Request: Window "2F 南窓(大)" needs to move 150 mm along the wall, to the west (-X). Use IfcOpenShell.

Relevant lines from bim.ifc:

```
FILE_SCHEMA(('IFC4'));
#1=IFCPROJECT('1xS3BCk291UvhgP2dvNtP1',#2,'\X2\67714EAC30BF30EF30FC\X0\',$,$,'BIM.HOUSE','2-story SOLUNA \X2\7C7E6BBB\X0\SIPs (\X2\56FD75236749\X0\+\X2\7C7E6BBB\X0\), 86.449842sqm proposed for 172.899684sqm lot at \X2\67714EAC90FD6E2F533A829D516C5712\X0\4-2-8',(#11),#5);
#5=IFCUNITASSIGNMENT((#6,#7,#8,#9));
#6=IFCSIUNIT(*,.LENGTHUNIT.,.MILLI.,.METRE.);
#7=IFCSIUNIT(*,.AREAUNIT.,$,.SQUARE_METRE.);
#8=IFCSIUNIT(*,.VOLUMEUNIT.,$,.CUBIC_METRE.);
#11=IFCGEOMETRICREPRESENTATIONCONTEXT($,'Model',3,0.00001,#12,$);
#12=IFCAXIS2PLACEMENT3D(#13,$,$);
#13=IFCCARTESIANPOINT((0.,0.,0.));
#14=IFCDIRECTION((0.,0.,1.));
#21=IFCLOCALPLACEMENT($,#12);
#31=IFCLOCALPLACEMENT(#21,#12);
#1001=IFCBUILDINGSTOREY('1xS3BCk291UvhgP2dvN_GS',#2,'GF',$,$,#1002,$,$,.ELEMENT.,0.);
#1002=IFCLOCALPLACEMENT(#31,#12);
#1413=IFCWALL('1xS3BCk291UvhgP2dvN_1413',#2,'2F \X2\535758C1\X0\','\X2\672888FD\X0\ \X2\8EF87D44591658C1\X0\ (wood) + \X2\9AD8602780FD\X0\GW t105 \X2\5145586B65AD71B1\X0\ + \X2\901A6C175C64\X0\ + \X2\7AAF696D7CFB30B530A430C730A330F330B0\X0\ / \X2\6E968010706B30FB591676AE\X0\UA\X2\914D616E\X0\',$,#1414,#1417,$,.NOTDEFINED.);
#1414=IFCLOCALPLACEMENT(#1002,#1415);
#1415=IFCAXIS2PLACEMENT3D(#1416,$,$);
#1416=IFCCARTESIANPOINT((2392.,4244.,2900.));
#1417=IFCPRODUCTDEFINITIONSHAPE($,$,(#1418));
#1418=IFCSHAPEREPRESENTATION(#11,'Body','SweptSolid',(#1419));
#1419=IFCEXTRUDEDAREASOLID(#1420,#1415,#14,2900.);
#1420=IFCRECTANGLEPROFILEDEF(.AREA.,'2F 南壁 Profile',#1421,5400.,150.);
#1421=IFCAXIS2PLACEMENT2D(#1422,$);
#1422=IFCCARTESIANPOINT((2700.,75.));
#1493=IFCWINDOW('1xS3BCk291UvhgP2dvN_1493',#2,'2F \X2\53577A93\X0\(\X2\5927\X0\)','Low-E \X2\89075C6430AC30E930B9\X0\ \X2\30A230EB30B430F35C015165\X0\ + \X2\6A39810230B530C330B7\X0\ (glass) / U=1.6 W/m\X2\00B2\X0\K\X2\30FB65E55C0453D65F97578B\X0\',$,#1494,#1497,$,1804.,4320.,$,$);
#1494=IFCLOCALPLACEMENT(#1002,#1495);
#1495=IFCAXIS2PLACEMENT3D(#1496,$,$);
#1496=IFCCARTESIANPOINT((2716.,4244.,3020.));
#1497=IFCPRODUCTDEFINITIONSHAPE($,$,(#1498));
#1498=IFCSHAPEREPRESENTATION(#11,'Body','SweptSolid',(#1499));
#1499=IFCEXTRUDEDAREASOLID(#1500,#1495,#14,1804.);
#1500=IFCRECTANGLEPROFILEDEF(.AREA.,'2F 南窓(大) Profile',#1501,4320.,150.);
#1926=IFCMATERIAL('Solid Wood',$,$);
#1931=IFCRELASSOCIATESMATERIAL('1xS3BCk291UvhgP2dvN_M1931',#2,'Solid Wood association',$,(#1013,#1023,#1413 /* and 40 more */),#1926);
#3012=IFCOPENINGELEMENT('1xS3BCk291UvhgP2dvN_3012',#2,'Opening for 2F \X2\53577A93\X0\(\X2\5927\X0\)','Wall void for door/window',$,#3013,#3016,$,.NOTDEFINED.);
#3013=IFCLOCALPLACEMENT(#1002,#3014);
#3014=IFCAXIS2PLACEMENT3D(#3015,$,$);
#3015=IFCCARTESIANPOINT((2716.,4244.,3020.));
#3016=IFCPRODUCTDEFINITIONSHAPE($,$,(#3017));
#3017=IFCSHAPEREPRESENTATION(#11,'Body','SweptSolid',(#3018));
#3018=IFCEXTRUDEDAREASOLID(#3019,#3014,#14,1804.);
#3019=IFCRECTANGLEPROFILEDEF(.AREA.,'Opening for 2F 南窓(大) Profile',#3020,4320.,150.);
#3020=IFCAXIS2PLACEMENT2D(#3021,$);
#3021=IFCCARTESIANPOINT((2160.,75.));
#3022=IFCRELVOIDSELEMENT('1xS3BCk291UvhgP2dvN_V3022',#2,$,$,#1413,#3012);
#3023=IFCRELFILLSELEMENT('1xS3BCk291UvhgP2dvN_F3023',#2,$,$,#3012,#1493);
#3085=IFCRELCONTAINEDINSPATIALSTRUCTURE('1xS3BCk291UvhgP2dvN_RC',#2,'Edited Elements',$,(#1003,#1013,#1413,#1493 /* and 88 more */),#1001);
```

```python
import ifcopenshell
import ifcopenshell.api.geometry
import ifcopenshell.util.placement
import ifcopenshell.util.unit

model = ifcopenshell.open("bim.ifc")
unit_scale = ifcopenshell.util.unit.calculate_unit_scale(model)

window = model.by_guid("1xS3BCk291UvhgP2dvN_1493")
opening = window.FillsVoids[0].RelatingOpeningElement
wall = opening.VoidsElements[0].RelatingBuildingElement

wall_matrix = ifcopenshell.util.placement.get_local_placement(wall.ObjectPlacement)
shift = wall_matrix[:3, 0] * -0.15 / unit_scale
before = ifcopenshell.util.placement.get_local_placement(window.ObjectPlacement)[:3, 3].copy()

# The window is not placed relative to its opening, so move both.
for product in (opening, window):
    matrix = ifcopenshell.util.placement.get_local_placement(product.ObjectPlacement)
    matrix[:3, 3] += shift
    ifcopenshell.api.geometry.edit_object_placement(model, product=product, matrix=matrix, is_si=False)

after = ifcopenshell.util.placement.get_local_placement(window.ObjectPlacement)[:3, 3]
print("window moved by", (after - before).round(3) + 0.0)

model.write("bim-out.ifc")
```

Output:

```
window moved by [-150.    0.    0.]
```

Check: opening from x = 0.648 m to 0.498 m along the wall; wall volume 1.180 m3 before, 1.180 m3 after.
